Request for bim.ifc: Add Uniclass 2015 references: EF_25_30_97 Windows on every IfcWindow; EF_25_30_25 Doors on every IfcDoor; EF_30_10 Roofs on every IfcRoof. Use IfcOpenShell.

First a look at what the model holds.

```python
import ifcopenshell

model = ifcopenshell.open("bim.ifc")
print(model.schema)
print("classifications:", [c.Name for c in model.by_type("IfcClassification")])
for ifc_class in ("IfcDoor", "IfcRoof", "IfcStair", "IfcWall", "IfcWindow"):
    print(ifc_class, len(model.by_type(ifc_class)))
```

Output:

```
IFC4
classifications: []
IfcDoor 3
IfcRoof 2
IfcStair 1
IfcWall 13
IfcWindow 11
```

```python
import ifcopenshell
import ifcopenshell.api.classification

model = ifcopenshell.open("bim.ifc")

system = ifcopenshell.api.classification.add_classification(model, classification="Uniclass 2015")

codes = {
    "IfcWindow": ("EF_25_30_97", "Windows"),
    "IfcDoor": ("EF_25_30_25", "Doors"),
    "IfcRoof": ("EF_30_10", "Roofs"),
}
for ifc_class, (code, name) in codes.items():
    products = model.by_type(ifc_class)
    ifcopenshell.api.classification.add_reference(
        model, products=products, classification=system, identification=code, name=name
    )
    print(code, len(products))

model.write("bim_updated.ifc")
```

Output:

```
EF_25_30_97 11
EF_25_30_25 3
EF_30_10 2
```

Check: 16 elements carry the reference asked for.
